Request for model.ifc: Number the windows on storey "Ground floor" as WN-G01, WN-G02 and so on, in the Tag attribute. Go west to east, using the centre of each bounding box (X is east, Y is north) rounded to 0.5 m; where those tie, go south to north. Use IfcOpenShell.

First a look at what the model holds.

```python
import ifcopenshell
import ifcopenshell.util.element
import ifcopenshell.util.placement

model = ifcopenshell.open("model.ifc")
print(model.schema)
storey = next(s for s in model.by_type("IfcBuildingStorey") if s.Name == "Ground floor")
windows = [e for e in ifcopenshell.util.element.get_decomposition(storey) if e.is_a("IfcWindow")]
for e in sorted(windows, key=lambda e: e.id()):
    origin = ifcopenshell.util.placement.get_local_placement(e.ObjectPlacement)[:3, 3]
    print(e.id(), e.Tag, e.Name, origin.round(2) + 0.0, sep=" | ")
```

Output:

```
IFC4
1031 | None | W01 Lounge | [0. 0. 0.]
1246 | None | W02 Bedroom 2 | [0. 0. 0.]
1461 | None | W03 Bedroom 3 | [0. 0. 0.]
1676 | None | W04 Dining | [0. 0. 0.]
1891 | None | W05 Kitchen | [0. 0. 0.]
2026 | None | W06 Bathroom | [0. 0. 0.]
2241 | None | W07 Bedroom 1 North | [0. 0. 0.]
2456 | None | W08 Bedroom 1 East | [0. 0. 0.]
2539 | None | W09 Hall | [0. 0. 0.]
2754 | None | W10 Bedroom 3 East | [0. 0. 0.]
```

```python
import ifcopenshell
import ifcopenshell.geom
import ifcopenshell.util.element
import ifcopenshell.util.shape

model = ifcopenshell.open("model.ifc")
settings = ifcopenshell.geom.settings()
settings.set("use-world-coords", True)


def centre(element):
    shape = ifcopenshell.geom.create_shape(settings, element)
    return ifcopenshell.util.shape.get_bbox_centroid(shape.geometry)


storey = next(s for s in model.by_type("IfcBuildingStorey") if s.Name == "Ground floor")
windows = [e for e in ifcopenshell.util.element.get_decomposition(storey) if e.is_a("IfcWindow")]

# Insertion points can sit at a corner or the storey origin, so sort by the geometry (in metres).
centres = {e: centre(e) for e in windows}
windows.sort(key=lambda e: (round(centres[e][0] / 0.5), centres[e][1]))

for i, e in enumerate(windows, start=1):
    number = f"WN-G{i:02d}"
    e.Tag = number
    print(e.id(), number)

model.write("model_edited.ifc")
```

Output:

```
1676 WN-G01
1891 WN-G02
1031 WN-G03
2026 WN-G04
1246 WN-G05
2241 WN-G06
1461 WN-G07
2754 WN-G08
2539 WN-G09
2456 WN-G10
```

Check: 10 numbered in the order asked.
